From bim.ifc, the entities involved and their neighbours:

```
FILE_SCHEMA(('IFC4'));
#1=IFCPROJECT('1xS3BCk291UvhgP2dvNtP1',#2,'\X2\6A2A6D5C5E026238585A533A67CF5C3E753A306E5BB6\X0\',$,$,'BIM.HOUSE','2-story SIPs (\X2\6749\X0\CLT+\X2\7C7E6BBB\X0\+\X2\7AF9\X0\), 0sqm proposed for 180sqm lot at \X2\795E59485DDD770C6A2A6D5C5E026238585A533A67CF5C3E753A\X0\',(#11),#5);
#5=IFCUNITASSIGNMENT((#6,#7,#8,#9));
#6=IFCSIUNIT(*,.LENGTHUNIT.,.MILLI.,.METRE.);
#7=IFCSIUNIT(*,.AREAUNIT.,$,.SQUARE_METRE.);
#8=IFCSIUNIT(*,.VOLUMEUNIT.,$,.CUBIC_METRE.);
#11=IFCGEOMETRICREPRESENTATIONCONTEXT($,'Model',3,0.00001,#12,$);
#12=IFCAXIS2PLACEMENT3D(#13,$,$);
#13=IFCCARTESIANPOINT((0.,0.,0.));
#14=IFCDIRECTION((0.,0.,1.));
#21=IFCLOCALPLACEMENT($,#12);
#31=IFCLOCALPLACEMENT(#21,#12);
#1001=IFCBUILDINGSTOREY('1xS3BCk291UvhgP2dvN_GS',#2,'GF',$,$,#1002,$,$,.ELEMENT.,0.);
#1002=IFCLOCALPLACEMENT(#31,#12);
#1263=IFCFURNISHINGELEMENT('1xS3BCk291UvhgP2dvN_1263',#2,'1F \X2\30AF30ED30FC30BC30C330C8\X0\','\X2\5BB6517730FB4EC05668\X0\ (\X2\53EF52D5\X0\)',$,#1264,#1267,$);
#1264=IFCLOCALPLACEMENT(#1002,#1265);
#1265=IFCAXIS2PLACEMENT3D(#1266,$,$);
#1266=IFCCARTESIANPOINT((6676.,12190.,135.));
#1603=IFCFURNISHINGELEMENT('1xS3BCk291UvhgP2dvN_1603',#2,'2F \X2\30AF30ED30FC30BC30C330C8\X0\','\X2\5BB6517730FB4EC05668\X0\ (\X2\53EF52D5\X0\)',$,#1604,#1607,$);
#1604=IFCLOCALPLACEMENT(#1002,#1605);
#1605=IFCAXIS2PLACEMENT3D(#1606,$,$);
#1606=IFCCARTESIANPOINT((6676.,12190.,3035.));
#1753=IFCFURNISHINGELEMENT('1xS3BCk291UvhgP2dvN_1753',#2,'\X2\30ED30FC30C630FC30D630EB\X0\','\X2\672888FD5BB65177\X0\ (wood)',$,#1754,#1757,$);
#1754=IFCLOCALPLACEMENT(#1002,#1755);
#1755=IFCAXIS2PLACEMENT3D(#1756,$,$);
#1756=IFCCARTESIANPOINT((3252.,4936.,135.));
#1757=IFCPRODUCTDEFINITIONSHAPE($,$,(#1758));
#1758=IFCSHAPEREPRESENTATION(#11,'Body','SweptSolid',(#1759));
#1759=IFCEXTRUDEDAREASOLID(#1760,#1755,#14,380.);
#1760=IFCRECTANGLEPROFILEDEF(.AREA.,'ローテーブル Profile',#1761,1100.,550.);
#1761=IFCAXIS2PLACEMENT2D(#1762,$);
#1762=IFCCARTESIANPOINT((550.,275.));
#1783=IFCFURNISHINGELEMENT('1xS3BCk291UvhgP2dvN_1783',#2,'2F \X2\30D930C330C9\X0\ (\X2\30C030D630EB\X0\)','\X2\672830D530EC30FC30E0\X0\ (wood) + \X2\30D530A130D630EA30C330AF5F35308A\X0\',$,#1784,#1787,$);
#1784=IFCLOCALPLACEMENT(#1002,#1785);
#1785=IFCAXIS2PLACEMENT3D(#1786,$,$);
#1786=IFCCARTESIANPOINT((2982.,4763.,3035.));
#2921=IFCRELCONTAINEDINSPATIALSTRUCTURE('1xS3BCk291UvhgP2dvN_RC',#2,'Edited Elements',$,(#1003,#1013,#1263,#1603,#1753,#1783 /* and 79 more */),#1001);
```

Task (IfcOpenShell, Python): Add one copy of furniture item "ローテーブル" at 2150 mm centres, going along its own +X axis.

```python
import ifcopenshell
import ifcopenshell.api.geometry
import ifcopenshell.api.root
import ifcopenshell.util.element
import ifcopenshell.util.placement
import ifcopenshell.util.unit

model = ifcopenshell.open("bim.ifc")
unit_scale = ifcopenshell.util.unit.calculate_unit_scale(model)


def reuse_history(source, copy):
    """copy_class also copies each property set's owner history, people and application; keep the originals."""
    for rel in copy.IsDefinedBy:
        if rel.is_a("IfcRelDefinesByProperties") and (history := rel.RelatingPropertyDefinition.OwnerHistory):
            rel.RelatingPropertyDefinition.OwnerHistory = source.OwnerHistory
            ifcopenshell.util.element.remove_deep2(model, history)


source = model.by_id(1753)
base = ifcopenshell.util.placement.get_local_placement(source.ObjectPlacement)
step = base[:3, 0] * 2.15 / unit_scale

for i in range(1, 2):
    copy = ifcopenshell.api.root.copy_class(model, product=source)
    copy.Representation = ifcopenshell.util.element.copy_deep(
        model, source.Representation, exclude=["IfcGeometricRepresentationContext", "IfcRepresentationMap"]
    )
    reuse_history(source, copy)
    matrix = base.copy()
    matrix[:3, 3] += i * step
    print("added at", matrix[:3, 3].round(3) + 0.0)
    ifcopenshell.api.geometry.edit_object_placement(model, product=copy, matrix=matrix, is_si=False)

model.write("bim-out.ifc")
```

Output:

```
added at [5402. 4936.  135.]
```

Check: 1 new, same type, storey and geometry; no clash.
